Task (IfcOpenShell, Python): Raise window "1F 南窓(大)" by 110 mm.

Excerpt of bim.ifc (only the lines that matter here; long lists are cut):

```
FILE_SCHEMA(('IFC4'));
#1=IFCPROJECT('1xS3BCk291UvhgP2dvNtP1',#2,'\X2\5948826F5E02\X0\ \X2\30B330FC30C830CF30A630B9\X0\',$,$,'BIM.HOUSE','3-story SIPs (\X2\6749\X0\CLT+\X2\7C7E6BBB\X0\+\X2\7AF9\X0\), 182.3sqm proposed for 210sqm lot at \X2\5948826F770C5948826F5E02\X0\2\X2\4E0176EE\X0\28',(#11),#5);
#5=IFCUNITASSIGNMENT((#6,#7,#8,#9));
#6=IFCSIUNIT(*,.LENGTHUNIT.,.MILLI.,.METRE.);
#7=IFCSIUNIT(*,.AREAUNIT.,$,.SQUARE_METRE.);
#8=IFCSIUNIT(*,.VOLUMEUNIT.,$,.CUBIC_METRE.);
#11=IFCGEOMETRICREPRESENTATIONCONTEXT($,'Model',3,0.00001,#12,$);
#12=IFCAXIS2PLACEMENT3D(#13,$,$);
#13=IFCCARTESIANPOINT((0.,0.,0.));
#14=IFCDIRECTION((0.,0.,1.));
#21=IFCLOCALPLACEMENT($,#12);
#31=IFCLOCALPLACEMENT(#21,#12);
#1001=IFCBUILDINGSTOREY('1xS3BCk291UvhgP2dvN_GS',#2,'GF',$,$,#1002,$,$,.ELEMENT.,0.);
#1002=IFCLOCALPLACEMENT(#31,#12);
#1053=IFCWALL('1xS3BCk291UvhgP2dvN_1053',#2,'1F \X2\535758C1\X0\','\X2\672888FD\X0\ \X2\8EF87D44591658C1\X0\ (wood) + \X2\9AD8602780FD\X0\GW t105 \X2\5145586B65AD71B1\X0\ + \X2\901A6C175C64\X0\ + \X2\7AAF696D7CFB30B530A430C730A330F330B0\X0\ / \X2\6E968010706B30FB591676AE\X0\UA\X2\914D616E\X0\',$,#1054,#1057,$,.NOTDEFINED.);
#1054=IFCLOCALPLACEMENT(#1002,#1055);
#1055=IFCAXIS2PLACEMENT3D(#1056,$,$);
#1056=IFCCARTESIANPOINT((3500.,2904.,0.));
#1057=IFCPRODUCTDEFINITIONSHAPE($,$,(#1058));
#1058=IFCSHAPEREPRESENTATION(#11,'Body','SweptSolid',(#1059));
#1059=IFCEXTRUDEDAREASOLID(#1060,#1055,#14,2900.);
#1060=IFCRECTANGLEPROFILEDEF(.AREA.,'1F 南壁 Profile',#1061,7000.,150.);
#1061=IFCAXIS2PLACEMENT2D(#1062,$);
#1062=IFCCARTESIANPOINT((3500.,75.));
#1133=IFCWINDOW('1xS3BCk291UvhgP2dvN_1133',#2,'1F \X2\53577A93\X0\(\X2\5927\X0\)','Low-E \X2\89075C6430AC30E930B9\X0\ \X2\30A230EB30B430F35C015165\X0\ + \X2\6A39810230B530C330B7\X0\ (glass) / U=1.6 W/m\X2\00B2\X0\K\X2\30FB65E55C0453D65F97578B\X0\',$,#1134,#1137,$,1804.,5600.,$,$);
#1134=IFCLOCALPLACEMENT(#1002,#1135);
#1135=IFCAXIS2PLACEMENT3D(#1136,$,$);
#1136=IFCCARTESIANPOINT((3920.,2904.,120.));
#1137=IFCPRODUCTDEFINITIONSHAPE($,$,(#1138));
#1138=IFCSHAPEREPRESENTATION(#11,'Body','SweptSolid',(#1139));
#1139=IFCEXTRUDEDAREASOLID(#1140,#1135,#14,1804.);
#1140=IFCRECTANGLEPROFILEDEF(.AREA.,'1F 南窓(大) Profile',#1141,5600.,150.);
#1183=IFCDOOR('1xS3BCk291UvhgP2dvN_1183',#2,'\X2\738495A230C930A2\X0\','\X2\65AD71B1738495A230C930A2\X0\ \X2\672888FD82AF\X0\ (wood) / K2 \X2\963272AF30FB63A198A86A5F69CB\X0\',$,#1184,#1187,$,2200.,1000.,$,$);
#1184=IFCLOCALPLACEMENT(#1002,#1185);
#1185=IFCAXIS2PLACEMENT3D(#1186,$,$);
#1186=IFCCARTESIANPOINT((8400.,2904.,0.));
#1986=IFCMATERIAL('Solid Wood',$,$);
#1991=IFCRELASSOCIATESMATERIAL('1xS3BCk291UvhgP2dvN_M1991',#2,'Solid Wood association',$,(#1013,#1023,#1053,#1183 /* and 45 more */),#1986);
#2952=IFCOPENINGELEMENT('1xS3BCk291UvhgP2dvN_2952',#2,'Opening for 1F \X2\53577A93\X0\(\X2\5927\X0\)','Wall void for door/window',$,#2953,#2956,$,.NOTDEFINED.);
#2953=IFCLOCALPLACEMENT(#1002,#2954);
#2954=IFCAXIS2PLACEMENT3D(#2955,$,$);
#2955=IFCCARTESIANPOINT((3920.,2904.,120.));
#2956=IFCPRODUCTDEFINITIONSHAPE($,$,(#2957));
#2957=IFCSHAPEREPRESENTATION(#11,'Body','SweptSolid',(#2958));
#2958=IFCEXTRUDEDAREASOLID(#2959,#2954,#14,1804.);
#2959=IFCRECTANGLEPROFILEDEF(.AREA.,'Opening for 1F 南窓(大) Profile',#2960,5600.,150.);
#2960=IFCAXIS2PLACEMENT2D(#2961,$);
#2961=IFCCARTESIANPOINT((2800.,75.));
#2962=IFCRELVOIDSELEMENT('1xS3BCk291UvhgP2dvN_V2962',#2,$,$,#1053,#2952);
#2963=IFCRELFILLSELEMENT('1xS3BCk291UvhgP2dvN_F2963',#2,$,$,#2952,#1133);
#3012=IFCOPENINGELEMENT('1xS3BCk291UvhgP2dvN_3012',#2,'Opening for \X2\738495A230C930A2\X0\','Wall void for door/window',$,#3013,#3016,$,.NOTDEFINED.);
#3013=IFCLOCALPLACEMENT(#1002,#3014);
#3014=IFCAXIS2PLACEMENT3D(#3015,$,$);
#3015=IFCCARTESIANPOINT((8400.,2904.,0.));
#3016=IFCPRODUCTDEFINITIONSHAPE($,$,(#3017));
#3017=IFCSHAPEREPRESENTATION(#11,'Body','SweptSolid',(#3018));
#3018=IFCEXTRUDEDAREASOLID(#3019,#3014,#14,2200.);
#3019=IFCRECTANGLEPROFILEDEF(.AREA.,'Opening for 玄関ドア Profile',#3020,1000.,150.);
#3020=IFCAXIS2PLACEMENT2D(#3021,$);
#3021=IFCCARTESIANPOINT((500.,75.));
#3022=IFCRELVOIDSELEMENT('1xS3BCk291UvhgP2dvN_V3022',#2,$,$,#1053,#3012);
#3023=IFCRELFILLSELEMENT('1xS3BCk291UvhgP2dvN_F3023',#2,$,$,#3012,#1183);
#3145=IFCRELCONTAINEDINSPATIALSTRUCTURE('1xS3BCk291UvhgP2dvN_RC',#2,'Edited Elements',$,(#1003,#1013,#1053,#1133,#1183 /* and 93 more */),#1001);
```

```python
import numpy as np
import ifcopenshell
import ifcopenshell.api.geometry
import ifcopenshell.util.placement
import ifcopenshell.util.unit

model = ifcopenshell.open("bim.ifc")
unit_scale = ifcopenshell.util.unit.calculate_unit_scale(model)

window = model.by_id(1133)
opening = window.FillsVoids[0].RelatingOpeningElement
dz = 0.11 / unit_scale

shift = np.array([0.0, 0.0, dz])
# The window is not placed relative to its opening, so move both.
for product in (opening, window):
    matrix = ifcopenshell.util.placement.get_local_placement(product.ObjectPlacement)
    matrix[:3, 3] += shift
    ifcopenshell.api.geometry.edit_object_placement(model, product=product, matrix=matrix, is_si=False)

print(f"moved by {dz * unit_scale:+.3f} m")

model.write("bim_updated.ifc")
```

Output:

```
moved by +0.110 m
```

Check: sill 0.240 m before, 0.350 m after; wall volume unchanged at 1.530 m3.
